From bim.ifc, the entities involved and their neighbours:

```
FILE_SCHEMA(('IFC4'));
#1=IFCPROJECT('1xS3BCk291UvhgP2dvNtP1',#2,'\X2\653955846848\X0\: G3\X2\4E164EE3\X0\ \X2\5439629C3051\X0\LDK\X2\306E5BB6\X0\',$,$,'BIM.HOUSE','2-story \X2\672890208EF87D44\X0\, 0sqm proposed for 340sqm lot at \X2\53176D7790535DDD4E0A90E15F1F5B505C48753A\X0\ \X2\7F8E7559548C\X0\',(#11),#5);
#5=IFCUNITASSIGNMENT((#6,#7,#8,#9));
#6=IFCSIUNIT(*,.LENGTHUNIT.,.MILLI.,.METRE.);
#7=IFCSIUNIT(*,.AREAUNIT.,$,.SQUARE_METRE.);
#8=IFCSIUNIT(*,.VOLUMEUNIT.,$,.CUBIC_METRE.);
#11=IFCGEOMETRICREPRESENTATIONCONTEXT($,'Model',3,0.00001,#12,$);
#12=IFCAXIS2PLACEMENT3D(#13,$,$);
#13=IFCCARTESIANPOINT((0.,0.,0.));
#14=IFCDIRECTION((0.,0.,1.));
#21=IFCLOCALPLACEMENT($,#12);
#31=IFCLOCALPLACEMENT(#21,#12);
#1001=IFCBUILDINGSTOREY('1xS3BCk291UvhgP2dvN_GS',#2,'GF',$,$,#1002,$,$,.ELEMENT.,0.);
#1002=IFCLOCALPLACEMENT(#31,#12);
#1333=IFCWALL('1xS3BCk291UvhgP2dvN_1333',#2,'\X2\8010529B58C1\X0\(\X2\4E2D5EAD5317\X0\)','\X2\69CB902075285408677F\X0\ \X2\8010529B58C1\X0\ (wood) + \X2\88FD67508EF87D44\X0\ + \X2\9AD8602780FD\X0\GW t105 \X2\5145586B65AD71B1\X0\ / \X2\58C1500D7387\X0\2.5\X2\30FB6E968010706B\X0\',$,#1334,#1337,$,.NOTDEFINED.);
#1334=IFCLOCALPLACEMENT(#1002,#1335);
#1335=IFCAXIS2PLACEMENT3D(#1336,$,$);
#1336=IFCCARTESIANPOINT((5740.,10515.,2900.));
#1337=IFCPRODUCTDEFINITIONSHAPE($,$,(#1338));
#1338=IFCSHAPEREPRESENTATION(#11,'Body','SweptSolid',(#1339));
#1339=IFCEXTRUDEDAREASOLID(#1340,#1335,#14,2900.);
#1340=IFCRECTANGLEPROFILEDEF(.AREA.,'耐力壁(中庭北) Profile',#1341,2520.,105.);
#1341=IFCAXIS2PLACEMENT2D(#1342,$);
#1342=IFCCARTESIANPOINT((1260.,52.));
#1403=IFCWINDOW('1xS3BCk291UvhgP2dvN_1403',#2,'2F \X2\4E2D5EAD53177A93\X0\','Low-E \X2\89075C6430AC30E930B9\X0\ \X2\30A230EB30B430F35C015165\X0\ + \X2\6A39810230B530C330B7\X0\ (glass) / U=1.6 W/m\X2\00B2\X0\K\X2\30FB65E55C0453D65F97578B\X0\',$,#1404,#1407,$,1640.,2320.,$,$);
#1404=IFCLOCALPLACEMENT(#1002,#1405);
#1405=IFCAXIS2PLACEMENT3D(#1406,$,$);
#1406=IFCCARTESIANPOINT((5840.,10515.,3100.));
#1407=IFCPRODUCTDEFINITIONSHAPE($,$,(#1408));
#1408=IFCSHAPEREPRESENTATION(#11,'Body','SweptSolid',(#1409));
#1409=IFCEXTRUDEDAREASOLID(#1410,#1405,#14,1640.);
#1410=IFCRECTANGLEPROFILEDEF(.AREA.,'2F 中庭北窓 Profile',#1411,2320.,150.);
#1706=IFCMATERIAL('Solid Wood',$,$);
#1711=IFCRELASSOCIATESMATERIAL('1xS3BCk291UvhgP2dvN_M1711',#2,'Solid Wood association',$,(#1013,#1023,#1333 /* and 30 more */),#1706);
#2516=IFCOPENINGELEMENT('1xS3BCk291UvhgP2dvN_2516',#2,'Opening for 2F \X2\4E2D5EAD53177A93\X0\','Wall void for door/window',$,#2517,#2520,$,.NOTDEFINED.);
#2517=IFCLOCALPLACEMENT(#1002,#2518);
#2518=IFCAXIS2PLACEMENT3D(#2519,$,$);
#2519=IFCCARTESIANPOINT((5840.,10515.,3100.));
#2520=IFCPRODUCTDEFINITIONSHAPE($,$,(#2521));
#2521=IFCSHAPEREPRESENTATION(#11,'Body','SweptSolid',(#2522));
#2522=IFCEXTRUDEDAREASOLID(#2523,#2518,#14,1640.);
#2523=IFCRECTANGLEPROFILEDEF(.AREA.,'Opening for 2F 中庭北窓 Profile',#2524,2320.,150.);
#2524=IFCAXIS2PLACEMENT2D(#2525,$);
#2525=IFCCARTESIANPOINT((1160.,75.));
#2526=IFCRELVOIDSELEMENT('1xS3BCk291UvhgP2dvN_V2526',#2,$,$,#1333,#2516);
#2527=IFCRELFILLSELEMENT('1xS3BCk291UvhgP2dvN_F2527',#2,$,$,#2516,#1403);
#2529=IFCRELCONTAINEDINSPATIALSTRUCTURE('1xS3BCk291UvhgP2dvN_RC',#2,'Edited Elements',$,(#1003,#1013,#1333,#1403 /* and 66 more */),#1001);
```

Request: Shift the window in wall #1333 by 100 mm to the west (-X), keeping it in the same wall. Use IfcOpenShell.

```python
import ifcopenshell
import ifcopenshell.api.geometry
import ifcopenshell.util.placement
import ifcopenshell.util.unit

model = ifcopenshell.open("bim.ifc")
unit_scale = ifcopenshell.util.unit.calculate_unit_scale(model)

window = model.by_id(1403)
opening = window.FillsVoids[0].RelatingOpeningElement
wall = opening.VoidsElements[0].RelatingBuildingElement

wall_matrix = ifcopenshell.util.placement.get_local_placement(wall.ObjectPlacement)
shift = wall_matrix[:3, 0] * -0.1 / unit_scale
before = ifcopenshell.util.placement.get_local_placement(window.ObjectPlacement)[:3, 3].copy()

# The window is not placed relative to its opening, so move both.
for product in (opening, window):
    matrix = ifcopenshell.util.placement.get_local_placement(product.ObjectPlacement)
    matrix[:3, 3] += shift
    ifcopenshell.api.geometry.edit_object_placement(model, product=product, matrix=matrix, is_si=False)

after = ifcopenshell.util.placement.get_local_placement(window.ObjectPlacement)[:3, 3]
print("window moved by", (after - before).round(3) + 0.0)

model.write("bim_updated.ifc")
```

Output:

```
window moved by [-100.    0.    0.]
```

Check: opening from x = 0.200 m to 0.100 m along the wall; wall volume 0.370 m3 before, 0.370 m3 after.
